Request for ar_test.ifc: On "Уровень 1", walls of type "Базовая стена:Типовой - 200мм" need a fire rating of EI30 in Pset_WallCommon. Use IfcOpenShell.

First a look at what the model holds.

```python
import ifcopenshell
import ifcopenshell.util.element

model = ifcopenshell.open("ar_test.ifc")
print(model.schema)
storey = next(s for s in model.by_type("IfcBuildingStorey") if s.Name == "Уровень 1")
walls = [e for e in ifcopenshell.util.element.get_decomposition(storey) if e.is_a("IfcWall")]
seen = {}
for e in walls:
    element_type = ifcopenshell.util.element.get_type(e)
    key = (element_type.Name if element_type != e and element_type else None, ifcopenshell.util.element.get_pset(e, "Pset_WallCommon", "FireRating"))
    seen[key] = seen.get(key, 0) + 1
for (name, value), count in sorted(seen.items(), key=str):
    print(count, "x", name, "|", value)
```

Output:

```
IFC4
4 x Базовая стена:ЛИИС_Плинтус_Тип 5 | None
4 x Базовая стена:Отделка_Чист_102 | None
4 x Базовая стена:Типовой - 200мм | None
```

```python
import ifcopenshell
import ifcopenshell.api.pset
import ifcopenshell.util.element

model = ifcopenshell.open("ar_test.ifc")

storey = next(s for s in model.by_type("IfcBuildingStorey") if s.Name == "Уровень 1")
walls = [e for e in ifcopenshell.util.element.get_decomposition(storey) if e.is_a("IfcWall")]

count = 0
for e in walls:
    element_type = ifcopenshell.util.element.get_type(e)
    if element_type in (None, e) or element_type.Name != "Базовая стена:Типовой - 200мм":
        continue
    # add_pset returns the element's existing set when there is one.
    pset = ifcopenshell.api.pset.add_pset(model, product=e, name="Pset_WallCommon")
    ifcopenshell.api.pset.edit_pset(model, pset=pset, properties={"FireRating": "EI30"})
    count += 1

print(count, "walls updated")

model.write("ar_test-out.ifc")
```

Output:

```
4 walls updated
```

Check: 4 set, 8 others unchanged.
